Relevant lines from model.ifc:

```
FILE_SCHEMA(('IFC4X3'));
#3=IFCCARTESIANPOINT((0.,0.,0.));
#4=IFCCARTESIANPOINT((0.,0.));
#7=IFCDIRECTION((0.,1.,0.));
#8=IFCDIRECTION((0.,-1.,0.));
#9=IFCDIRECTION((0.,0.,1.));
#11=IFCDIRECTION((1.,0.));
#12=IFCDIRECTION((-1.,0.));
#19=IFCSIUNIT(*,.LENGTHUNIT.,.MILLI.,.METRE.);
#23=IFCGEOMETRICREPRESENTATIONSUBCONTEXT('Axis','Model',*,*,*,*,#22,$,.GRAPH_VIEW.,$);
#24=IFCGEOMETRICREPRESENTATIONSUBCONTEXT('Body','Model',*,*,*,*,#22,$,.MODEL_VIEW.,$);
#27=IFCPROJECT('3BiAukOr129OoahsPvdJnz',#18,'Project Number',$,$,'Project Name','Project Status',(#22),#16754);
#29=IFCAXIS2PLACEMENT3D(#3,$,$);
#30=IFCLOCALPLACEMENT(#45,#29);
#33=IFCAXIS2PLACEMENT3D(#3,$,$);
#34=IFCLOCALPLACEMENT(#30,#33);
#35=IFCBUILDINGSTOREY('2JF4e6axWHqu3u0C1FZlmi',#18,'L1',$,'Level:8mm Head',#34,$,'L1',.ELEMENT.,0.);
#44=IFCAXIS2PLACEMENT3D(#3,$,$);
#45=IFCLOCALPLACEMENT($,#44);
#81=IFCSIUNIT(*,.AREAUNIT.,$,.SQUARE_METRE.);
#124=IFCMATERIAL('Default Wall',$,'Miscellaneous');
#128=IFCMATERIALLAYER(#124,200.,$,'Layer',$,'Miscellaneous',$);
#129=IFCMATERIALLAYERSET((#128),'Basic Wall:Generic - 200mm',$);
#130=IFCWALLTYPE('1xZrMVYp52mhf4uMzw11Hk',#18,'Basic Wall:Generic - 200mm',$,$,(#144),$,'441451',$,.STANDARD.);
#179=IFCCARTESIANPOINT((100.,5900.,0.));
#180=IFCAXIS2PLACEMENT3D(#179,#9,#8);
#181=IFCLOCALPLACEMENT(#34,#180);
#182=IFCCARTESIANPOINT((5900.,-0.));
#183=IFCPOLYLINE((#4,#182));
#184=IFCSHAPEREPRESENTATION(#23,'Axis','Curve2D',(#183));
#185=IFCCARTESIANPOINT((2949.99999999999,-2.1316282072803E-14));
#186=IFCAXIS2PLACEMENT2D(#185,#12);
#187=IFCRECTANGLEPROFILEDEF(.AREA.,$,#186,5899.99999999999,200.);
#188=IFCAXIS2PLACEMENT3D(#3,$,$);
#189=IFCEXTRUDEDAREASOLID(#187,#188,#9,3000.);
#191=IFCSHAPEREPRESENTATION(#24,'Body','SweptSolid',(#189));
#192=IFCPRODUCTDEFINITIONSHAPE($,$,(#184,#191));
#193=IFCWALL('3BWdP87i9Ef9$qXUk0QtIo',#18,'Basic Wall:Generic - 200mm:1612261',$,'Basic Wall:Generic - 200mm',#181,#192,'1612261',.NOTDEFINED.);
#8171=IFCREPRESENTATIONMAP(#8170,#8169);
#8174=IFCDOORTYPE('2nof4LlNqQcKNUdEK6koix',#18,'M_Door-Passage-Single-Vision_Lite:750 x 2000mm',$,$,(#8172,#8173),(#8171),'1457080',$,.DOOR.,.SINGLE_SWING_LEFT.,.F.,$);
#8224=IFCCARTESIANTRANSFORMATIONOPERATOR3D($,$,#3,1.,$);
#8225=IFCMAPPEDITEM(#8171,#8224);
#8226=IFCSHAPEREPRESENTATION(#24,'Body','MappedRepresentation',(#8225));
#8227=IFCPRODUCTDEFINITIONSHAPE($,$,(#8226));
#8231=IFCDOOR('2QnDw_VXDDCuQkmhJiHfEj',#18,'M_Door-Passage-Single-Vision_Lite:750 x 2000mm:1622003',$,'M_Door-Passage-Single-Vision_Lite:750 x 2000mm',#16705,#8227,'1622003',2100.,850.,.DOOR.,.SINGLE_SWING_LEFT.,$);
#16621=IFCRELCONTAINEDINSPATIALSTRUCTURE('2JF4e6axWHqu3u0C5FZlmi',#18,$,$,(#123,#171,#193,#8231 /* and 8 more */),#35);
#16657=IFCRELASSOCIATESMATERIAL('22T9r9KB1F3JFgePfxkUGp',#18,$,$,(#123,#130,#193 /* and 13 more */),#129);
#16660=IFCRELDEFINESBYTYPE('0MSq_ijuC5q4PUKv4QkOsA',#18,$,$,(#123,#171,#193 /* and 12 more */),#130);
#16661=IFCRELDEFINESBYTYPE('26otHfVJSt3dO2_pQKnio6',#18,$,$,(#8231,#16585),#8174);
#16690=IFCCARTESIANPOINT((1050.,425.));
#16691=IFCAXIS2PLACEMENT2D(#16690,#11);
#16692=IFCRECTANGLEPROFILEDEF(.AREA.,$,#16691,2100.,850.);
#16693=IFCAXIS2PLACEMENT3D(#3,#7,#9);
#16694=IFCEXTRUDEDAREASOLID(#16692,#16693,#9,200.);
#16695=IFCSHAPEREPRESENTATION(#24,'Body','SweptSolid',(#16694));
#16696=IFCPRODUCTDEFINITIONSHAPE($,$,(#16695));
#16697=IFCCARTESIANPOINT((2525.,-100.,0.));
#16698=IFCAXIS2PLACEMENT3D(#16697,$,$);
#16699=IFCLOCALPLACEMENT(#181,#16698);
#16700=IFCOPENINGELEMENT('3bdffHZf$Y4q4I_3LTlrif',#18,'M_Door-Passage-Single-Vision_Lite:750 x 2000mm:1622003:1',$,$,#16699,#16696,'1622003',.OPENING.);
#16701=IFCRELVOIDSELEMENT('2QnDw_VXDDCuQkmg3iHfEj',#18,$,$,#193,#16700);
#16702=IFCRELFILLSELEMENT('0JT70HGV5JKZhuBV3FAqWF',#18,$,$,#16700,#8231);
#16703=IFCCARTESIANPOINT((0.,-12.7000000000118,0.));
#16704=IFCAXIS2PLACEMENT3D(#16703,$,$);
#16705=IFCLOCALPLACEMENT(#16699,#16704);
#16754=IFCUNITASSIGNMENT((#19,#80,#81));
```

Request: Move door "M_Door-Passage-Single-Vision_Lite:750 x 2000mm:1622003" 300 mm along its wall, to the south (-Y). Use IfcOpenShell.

```python
import ifcopenshell
import ifcopenshell.api.geometry
import ifcopenshell.util.placement

model = ifcopenshell.open("model.ifc")

door = model.by_id(8231)
opening = door.FillsVoids[0].RelatingOpeningElement
wall = opening.VoidsElements[0].RelatingBuildingElement

wall_matrix = ifcopenshell.util.placement.get_local_placement(wall.ObjectPlacement)
shift = wall_matrix[:3, 0] * 300.0
before = ifcopenshell.util.placement.get_local_placement(door.ObjectPlacement)[:3, 3].copy()

# The door is placed relative to its opening, so it follows when the opening moves.
matrix = ifcopenshell.util.placement.get_local_placement(opening.ObjectPlacement)
matrix[:3, 3] += shift
ifcopenshell.api.geometry.edit_object_placement(
    model, product=opening, matrix=matrix, is_si=False, should_transform_children=True
)

after = ifcopenshell.util.placement.get_local_placement(door.ObjectPlacement)[:3, 3]
print("door moved by", (after - before).round(3) + 0.0)

model.write("model-out.ifc")
```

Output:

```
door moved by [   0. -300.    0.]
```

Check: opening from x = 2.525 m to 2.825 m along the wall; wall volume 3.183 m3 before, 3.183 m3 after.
